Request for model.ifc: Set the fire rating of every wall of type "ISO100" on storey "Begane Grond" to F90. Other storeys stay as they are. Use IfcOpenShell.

First a look at what the model holds.

```python
import ifcopenshell
import ifcopenshell.util.element

model = ifcopenshell.open("model.ifc")
print(model.schema)
storey = next(s for s in model.by_type("IfcBuildingStorey") if s.Name == "Begane Grond")
walls = [e for e in ifcopenshell.util.element.get_decomposition(storey) if e.is_a("IfcWall")]
seen = {}
for e in walls:
    element_type = ifcopenshell.util.element.get_type(e)
    key = (element_type.Name if element_type != e and element_type else None, ifcopenshell.util.element.get_pset(e, "Pset_WallCommon", "FireRating"))
    seen[key] = seen.get(key, 0) + 1
for (name, value), count in sorted(seen.items(), key=str):
    print(count, "x", name, "|", value)
```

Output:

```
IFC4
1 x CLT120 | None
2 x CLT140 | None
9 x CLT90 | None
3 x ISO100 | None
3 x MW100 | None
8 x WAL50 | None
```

```python
import ifcopenshell
import ifcopenshell.api.pset
import ifcopenshell.util.element

model = ifcopenshell.open("model.ifc")

storey = next(s for s in model.by_type("IfcBuildingStorey") if s.Name == "Begane Grond")
walls = [e for e in ifcopenshell.util.element.get_decomposition(storey) if e.is_a("IfcWall")]

count = 0
for e in walls:
    element_type = ifcopenshell.util.element.get_type(e)
    if element_type in (None, e) or element_type.Name != "ISO100":
        continue
    # add_pset returns the element's existing set when there is one.
    pset = ifcopenshell.api.pset.add_pset(model, product=e, name="Pset_WallCommon")
    ifcopenshell.api.pset.edit_pset(model, pset=pset, properties={"FireRating": "F90"})
    count += 1

print(count, "walls updated")

model.write("model_v2.ifc")
```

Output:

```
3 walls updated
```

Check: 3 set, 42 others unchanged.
